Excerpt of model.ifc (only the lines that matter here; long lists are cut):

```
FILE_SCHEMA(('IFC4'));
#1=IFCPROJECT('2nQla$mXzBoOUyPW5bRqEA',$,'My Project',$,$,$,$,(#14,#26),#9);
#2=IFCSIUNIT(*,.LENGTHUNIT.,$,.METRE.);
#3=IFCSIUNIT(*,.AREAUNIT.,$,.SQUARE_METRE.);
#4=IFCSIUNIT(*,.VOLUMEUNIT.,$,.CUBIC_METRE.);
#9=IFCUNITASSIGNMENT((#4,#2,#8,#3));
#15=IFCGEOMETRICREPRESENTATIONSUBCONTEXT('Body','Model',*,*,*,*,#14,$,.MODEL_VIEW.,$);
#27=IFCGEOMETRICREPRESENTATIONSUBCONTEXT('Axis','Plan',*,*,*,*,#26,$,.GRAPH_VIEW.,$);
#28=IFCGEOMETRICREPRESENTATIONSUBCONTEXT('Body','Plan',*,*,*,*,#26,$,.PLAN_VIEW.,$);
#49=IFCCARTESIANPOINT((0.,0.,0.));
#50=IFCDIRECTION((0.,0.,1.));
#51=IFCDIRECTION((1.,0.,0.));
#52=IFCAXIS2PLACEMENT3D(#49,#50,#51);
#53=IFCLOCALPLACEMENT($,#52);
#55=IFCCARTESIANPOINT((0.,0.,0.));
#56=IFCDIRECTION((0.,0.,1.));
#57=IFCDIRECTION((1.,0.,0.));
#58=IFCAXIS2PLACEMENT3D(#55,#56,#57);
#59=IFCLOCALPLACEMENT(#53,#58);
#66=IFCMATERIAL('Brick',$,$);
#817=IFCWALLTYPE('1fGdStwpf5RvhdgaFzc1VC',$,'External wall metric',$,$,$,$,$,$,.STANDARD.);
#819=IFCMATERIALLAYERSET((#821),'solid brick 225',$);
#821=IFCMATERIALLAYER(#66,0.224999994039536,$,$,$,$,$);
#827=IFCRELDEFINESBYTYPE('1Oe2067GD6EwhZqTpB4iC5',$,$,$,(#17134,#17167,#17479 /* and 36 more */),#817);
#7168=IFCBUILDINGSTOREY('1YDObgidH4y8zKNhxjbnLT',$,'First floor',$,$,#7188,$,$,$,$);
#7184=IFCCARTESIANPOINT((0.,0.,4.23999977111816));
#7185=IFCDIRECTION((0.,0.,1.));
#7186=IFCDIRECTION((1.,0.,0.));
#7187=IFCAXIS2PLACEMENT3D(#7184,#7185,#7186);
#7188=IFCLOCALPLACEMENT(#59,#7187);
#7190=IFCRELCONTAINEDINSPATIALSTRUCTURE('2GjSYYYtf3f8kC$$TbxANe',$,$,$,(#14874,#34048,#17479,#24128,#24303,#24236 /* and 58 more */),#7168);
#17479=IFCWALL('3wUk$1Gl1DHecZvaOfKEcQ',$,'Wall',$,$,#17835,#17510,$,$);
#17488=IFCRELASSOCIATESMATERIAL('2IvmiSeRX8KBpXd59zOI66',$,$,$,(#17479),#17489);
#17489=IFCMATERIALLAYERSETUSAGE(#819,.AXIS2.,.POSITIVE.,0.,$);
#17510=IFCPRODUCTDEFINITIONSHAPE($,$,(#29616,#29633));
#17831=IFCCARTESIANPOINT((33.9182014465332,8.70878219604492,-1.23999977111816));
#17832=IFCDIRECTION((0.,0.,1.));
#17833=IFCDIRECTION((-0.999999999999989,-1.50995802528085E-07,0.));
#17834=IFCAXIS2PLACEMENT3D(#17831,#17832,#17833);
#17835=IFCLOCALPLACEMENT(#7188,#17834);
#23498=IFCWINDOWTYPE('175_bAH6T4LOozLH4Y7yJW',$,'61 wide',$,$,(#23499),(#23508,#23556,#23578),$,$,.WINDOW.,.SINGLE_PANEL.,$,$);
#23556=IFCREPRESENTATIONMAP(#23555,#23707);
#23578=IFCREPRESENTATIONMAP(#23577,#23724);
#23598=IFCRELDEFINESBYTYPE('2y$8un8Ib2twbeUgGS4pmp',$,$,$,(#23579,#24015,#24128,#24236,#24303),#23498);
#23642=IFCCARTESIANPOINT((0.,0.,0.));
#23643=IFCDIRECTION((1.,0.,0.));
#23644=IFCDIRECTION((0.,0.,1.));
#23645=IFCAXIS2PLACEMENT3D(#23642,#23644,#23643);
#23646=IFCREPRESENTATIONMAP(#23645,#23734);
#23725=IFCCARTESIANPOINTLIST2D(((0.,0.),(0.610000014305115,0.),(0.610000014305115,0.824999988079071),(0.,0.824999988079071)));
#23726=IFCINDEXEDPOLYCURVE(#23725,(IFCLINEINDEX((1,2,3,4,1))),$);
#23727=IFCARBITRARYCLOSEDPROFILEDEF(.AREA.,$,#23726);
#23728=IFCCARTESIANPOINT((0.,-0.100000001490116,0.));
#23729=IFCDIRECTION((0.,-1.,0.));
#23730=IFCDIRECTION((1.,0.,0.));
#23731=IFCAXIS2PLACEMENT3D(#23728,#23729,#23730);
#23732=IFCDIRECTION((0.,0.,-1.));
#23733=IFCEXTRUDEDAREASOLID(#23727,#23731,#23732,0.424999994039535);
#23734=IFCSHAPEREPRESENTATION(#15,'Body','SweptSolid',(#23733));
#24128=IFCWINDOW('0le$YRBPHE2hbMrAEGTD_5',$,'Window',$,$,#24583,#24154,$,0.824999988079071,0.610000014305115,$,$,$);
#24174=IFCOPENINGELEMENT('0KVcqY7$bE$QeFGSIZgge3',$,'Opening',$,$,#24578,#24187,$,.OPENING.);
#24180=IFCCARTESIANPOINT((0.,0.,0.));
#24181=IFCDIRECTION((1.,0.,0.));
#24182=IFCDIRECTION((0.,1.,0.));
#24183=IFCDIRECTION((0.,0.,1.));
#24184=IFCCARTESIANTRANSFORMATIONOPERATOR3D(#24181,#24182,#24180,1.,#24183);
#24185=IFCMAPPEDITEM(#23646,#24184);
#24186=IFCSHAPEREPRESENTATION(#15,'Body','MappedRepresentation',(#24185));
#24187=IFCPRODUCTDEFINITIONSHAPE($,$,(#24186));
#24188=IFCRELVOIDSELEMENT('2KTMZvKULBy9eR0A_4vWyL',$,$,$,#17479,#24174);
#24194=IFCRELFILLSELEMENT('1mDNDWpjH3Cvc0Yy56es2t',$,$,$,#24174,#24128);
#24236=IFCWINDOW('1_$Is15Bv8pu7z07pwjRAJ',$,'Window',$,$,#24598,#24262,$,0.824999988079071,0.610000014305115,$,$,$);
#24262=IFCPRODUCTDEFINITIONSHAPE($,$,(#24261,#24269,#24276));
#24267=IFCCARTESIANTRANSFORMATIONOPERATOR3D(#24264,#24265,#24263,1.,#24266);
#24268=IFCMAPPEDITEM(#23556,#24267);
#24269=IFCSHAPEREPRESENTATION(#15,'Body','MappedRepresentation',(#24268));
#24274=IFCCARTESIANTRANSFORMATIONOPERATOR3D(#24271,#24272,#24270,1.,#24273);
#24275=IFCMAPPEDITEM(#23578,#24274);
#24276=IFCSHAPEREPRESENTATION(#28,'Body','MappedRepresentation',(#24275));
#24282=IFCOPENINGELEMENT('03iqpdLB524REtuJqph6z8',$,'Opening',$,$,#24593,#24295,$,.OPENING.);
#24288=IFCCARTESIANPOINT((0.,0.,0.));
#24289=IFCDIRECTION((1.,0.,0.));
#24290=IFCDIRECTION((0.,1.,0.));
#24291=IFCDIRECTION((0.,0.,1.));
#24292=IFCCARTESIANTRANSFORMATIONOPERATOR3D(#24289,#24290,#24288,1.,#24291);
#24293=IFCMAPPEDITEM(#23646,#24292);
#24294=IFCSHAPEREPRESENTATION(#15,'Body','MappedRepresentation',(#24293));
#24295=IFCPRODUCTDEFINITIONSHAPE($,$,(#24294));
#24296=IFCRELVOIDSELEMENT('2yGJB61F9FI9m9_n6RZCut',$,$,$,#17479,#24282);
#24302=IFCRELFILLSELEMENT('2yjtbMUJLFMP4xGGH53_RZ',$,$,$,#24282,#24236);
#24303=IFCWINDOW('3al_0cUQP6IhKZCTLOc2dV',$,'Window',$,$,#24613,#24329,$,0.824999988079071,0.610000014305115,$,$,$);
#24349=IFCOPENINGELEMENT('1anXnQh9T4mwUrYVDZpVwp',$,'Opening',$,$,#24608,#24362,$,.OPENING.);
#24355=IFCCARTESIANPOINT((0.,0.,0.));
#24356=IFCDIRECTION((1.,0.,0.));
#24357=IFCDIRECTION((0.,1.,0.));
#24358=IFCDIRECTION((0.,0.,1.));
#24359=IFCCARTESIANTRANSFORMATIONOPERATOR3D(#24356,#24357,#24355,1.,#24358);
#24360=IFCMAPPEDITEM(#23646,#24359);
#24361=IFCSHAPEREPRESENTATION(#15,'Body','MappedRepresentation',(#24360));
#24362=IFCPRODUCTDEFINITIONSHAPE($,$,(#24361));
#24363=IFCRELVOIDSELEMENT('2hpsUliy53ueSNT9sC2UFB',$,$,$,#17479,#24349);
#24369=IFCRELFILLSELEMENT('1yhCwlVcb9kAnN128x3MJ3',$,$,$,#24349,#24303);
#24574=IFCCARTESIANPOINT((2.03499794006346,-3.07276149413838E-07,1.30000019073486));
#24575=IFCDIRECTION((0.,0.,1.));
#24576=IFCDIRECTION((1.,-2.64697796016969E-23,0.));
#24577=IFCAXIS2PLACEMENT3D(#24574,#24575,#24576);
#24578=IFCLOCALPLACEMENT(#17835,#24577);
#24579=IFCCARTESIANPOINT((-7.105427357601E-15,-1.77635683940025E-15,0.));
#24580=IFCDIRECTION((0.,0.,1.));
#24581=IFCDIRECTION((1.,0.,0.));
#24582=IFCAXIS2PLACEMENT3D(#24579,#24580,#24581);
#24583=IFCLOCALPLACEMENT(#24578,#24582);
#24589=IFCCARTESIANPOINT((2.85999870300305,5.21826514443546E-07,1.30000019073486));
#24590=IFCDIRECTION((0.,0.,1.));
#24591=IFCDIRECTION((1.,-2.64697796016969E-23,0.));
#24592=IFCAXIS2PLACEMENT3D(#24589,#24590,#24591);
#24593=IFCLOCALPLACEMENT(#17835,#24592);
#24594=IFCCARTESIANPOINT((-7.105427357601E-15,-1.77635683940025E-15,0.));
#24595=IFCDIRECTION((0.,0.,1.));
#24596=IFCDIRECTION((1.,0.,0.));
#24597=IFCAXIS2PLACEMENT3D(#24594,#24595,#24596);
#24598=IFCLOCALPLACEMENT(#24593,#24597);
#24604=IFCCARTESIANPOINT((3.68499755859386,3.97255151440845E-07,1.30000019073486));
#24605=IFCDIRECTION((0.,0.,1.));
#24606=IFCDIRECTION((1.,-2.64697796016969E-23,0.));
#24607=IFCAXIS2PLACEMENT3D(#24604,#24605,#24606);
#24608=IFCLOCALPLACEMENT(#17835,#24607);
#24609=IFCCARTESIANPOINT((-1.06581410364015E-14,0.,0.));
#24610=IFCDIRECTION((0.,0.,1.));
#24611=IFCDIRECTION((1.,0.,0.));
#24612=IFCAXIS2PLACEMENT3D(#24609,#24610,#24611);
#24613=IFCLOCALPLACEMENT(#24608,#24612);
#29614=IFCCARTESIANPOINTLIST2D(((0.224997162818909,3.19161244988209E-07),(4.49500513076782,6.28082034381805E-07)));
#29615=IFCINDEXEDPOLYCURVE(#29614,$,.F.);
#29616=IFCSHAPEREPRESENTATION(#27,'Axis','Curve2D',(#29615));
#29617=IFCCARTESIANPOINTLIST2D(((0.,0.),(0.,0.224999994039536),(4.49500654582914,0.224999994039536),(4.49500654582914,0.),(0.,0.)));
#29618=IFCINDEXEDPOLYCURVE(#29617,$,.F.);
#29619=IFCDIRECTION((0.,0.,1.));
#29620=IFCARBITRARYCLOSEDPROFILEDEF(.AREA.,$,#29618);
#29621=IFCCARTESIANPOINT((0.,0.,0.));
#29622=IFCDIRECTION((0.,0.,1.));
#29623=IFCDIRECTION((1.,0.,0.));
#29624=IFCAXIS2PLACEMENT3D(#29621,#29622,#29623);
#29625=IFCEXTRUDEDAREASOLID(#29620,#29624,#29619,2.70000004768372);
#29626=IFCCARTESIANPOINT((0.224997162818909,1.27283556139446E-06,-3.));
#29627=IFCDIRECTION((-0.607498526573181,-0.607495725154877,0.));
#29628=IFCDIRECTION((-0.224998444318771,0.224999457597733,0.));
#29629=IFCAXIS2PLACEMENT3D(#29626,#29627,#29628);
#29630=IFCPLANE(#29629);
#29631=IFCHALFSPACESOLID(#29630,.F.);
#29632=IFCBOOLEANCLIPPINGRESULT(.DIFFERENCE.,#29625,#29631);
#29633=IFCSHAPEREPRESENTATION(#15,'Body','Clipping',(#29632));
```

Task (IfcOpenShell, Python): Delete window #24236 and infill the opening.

```python
import ifcopenshell
import ifcopenshell.api.feature
import ifcopenshell.api.root
import ifcopenshell.geom
import ifcopenshell.util.shape

model = ifcopenshell.open("model.ifc")
settings = ifcopenshell.geom.settings()


def volume(element):
    """Net volume in cubic metres, openings subtracted."""
    shape = ifcopenshell.geom.create_shape(settings, element)
    return ifcopenshell.util.shape.get_volume(shape.geometry)


window = model.by_id(24236)
opening = window.FillsVoids[0].RelatingOpeningElement
wall = opening.VoidsElements[0].RelatingBuildingElement
before = volume(wall)

ifcopenshell.api.root.remove_product(model, product=window)
ifcopenshell.api.feature.remove_feature(model, feature=opening)

after = volume(wall)

print(f"wall volume {before:.3f} -> {after:.3f} m3")

model.write("model_edited.ifc")
```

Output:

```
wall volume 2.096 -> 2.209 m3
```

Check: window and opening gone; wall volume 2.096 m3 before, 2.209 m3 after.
